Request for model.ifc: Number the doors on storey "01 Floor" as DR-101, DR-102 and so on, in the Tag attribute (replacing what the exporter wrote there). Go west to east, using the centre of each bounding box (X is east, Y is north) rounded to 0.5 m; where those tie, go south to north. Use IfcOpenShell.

First a look at what the model holds.

```python
import ifcopenshell
import ifcopenshell.util.element
import ifcopenshell.util.placement

model = ifcopenshell.open("model.ifc")
print(model.schema)
storey = next(s for s in model.by_type("IfcBuildingStorey") if s.Name == "01 Floor")
doors = [e for e in ifcopenshell.util.element.get_decomposition(storey) if e.is_a("IfcDoor")]
for e in sorted(doors, key=lambda e: e.id()):
    origin = ifcopenshell.util.placement.get_local_placement(e.ObjectPlacement)[:3, 3]
    print(e.id(), e.Tag, e.Name, origin.round(2) + 0.0, sep=" | ")
```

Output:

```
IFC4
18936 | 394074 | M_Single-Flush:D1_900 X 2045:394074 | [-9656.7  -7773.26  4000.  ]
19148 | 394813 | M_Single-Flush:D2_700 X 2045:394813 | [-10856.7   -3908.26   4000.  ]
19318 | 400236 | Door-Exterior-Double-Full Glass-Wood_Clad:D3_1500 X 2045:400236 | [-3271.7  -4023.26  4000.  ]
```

```python
import ifcopenshell
import ifcopenshell.geom
import ifcopenshell.util.element
import ifcopenshell.util.shape

model = ifcopenshell.open("model.ifc")
settings = ifcopenshell.geom.settings()
settings.set("use-world-coords", True)


def centre(element):
    shape = ifcopenshell.geom.create_shape(settings, element)
    return ifcopenshell.util.shape.get_bbox_centroid(shape.geometry)


storey = next(s for s in model.by_type("IfcBuildingStorey") if s.Name == "01 Floor")
doors = [e for e in ifcopenshell.util.element.get_decomposition(storey) if e.is_a("IfcDoor")]

# Insertion points can sit at a corner or the storey origin, so sort by the geometry (in metres).
centres = {e: centre(e) for e in doors}
doors.sort(key=lambda e: (round(centres[e][0] / 0.5), centres[e][1]))

for i, e in enumerate(doors, start=1):
    number = f"DR-1{i:02d}"
    e.Tag = number
    print(e.id(), number)

model.write("model_updated.ifc")
```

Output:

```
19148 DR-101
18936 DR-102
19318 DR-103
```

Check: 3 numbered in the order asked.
